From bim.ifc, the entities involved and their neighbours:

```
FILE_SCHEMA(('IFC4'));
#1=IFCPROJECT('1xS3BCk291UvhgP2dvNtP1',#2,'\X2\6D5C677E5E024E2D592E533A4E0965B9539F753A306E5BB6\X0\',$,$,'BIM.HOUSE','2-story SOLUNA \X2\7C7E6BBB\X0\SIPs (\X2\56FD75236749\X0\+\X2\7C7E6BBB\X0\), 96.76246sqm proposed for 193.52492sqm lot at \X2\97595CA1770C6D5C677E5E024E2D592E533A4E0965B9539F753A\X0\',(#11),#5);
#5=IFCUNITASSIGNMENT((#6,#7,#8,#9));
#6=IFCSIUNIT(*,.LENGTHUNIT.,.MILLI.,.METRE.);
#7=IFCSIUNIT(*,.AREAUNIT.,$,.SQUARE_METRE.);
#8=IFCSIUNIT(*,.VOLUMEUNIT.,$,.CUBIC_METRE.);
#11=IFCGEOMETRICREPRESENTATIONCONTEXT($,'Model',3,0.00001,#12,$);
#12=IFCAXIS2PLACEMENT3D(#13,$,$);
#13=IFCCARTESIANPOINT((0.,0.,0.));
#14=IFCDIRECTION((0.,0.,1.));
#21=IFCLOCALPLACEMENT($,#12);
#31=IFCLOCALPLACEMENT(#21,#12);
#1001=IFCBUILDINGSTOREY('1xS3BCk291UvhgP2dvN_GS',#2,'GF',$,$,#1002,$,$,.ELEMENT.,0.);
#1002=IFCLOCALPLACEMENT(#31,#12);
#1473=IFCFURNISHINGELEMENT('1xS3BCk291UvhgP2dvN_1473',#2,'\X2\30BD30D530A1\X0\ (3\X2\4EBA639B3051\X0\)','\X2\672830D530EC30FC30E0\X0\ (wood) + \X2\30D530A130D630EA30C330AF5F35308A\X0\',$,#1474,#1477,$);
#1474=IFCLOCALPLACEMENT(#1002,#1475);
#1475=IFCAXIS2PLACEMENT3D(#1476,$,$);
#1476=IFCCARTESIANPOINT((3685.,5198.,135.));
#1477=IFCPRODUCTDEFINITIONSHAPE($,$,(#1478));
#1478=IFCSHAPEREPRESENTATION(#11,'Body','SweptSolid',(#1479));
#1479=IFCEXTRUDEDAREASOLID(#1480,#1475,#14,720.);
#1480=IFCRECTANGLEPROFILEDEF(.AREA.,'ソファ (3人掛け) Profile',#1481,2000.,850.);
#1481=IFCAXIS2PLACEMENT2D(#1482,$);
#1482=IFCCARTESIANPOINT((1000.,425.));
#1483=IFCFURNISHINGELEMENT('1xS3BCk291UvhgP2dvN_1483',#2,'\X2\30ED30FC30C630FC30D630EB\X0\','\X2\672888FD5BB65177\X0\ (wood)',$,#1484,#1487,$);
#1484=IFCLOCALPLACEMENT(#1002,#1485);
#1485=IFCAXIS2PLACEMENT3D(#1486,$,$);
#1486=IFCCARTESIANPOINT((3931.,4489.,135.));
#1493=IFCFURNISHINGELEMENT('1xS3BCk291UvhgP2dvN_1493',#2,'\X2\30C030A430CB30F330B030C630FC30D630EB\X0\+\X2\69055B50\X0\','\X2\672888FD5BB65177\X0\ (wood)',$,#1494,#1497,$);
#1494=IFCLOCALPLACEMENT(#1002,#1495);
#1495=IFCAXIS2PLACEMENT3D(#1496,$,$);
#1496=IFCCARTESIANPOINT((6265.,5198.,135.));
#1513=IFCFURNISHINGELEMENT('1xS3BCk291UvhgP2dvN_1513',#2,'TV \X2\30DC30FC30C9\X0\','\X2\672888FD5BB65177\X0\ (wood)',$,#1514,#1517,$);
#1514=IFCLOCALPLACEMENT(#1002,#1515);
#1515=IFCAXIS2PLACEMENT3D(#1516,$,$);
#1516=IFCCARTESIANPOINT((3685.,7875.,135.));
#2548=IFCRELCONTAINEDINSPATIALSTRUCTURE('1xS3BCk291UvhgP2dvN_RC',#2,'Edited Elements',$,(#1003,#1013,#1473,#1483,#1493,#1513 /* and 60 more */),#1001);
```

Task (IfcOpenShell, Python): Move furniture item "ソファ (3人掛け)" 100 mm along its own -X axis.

```python
import ifcopenshell
import ifcopenshell.api.geometry
import ifcopenshell.util.placement
import ifcopenshell.util.unit

model = ifcopenshell.open("bim.ifc")
unit_scale = ifcopenshell.util.unit.calculate_unit_scale(model)

item = model.by_guid("1xS3BCk291UvhgP2dvN_1473")
matrix = ifcopenshell.util.placement.get_local_placement(item.ObjectPlacement)
matrix[:3, 3] -= matrix[:3, 0] * 0.1 / unit_scale
ifcopenshell.api.geometry.edit_object_placement(model, product=item, matrix=matrix, is_si=False)

print(ifcopenshell.util.placement.get_local_placement(item.ObjectPlacement).round(3) + 0.0)

model.write("bim_rev.ifc")
```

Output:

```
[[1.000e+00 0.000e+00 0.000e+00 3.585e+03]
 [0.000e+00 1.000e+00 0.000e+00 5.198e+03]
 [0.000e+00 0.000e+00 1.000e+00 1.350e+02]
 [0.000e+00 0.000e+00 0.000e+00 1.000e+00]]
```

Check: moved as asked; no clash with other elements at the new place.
